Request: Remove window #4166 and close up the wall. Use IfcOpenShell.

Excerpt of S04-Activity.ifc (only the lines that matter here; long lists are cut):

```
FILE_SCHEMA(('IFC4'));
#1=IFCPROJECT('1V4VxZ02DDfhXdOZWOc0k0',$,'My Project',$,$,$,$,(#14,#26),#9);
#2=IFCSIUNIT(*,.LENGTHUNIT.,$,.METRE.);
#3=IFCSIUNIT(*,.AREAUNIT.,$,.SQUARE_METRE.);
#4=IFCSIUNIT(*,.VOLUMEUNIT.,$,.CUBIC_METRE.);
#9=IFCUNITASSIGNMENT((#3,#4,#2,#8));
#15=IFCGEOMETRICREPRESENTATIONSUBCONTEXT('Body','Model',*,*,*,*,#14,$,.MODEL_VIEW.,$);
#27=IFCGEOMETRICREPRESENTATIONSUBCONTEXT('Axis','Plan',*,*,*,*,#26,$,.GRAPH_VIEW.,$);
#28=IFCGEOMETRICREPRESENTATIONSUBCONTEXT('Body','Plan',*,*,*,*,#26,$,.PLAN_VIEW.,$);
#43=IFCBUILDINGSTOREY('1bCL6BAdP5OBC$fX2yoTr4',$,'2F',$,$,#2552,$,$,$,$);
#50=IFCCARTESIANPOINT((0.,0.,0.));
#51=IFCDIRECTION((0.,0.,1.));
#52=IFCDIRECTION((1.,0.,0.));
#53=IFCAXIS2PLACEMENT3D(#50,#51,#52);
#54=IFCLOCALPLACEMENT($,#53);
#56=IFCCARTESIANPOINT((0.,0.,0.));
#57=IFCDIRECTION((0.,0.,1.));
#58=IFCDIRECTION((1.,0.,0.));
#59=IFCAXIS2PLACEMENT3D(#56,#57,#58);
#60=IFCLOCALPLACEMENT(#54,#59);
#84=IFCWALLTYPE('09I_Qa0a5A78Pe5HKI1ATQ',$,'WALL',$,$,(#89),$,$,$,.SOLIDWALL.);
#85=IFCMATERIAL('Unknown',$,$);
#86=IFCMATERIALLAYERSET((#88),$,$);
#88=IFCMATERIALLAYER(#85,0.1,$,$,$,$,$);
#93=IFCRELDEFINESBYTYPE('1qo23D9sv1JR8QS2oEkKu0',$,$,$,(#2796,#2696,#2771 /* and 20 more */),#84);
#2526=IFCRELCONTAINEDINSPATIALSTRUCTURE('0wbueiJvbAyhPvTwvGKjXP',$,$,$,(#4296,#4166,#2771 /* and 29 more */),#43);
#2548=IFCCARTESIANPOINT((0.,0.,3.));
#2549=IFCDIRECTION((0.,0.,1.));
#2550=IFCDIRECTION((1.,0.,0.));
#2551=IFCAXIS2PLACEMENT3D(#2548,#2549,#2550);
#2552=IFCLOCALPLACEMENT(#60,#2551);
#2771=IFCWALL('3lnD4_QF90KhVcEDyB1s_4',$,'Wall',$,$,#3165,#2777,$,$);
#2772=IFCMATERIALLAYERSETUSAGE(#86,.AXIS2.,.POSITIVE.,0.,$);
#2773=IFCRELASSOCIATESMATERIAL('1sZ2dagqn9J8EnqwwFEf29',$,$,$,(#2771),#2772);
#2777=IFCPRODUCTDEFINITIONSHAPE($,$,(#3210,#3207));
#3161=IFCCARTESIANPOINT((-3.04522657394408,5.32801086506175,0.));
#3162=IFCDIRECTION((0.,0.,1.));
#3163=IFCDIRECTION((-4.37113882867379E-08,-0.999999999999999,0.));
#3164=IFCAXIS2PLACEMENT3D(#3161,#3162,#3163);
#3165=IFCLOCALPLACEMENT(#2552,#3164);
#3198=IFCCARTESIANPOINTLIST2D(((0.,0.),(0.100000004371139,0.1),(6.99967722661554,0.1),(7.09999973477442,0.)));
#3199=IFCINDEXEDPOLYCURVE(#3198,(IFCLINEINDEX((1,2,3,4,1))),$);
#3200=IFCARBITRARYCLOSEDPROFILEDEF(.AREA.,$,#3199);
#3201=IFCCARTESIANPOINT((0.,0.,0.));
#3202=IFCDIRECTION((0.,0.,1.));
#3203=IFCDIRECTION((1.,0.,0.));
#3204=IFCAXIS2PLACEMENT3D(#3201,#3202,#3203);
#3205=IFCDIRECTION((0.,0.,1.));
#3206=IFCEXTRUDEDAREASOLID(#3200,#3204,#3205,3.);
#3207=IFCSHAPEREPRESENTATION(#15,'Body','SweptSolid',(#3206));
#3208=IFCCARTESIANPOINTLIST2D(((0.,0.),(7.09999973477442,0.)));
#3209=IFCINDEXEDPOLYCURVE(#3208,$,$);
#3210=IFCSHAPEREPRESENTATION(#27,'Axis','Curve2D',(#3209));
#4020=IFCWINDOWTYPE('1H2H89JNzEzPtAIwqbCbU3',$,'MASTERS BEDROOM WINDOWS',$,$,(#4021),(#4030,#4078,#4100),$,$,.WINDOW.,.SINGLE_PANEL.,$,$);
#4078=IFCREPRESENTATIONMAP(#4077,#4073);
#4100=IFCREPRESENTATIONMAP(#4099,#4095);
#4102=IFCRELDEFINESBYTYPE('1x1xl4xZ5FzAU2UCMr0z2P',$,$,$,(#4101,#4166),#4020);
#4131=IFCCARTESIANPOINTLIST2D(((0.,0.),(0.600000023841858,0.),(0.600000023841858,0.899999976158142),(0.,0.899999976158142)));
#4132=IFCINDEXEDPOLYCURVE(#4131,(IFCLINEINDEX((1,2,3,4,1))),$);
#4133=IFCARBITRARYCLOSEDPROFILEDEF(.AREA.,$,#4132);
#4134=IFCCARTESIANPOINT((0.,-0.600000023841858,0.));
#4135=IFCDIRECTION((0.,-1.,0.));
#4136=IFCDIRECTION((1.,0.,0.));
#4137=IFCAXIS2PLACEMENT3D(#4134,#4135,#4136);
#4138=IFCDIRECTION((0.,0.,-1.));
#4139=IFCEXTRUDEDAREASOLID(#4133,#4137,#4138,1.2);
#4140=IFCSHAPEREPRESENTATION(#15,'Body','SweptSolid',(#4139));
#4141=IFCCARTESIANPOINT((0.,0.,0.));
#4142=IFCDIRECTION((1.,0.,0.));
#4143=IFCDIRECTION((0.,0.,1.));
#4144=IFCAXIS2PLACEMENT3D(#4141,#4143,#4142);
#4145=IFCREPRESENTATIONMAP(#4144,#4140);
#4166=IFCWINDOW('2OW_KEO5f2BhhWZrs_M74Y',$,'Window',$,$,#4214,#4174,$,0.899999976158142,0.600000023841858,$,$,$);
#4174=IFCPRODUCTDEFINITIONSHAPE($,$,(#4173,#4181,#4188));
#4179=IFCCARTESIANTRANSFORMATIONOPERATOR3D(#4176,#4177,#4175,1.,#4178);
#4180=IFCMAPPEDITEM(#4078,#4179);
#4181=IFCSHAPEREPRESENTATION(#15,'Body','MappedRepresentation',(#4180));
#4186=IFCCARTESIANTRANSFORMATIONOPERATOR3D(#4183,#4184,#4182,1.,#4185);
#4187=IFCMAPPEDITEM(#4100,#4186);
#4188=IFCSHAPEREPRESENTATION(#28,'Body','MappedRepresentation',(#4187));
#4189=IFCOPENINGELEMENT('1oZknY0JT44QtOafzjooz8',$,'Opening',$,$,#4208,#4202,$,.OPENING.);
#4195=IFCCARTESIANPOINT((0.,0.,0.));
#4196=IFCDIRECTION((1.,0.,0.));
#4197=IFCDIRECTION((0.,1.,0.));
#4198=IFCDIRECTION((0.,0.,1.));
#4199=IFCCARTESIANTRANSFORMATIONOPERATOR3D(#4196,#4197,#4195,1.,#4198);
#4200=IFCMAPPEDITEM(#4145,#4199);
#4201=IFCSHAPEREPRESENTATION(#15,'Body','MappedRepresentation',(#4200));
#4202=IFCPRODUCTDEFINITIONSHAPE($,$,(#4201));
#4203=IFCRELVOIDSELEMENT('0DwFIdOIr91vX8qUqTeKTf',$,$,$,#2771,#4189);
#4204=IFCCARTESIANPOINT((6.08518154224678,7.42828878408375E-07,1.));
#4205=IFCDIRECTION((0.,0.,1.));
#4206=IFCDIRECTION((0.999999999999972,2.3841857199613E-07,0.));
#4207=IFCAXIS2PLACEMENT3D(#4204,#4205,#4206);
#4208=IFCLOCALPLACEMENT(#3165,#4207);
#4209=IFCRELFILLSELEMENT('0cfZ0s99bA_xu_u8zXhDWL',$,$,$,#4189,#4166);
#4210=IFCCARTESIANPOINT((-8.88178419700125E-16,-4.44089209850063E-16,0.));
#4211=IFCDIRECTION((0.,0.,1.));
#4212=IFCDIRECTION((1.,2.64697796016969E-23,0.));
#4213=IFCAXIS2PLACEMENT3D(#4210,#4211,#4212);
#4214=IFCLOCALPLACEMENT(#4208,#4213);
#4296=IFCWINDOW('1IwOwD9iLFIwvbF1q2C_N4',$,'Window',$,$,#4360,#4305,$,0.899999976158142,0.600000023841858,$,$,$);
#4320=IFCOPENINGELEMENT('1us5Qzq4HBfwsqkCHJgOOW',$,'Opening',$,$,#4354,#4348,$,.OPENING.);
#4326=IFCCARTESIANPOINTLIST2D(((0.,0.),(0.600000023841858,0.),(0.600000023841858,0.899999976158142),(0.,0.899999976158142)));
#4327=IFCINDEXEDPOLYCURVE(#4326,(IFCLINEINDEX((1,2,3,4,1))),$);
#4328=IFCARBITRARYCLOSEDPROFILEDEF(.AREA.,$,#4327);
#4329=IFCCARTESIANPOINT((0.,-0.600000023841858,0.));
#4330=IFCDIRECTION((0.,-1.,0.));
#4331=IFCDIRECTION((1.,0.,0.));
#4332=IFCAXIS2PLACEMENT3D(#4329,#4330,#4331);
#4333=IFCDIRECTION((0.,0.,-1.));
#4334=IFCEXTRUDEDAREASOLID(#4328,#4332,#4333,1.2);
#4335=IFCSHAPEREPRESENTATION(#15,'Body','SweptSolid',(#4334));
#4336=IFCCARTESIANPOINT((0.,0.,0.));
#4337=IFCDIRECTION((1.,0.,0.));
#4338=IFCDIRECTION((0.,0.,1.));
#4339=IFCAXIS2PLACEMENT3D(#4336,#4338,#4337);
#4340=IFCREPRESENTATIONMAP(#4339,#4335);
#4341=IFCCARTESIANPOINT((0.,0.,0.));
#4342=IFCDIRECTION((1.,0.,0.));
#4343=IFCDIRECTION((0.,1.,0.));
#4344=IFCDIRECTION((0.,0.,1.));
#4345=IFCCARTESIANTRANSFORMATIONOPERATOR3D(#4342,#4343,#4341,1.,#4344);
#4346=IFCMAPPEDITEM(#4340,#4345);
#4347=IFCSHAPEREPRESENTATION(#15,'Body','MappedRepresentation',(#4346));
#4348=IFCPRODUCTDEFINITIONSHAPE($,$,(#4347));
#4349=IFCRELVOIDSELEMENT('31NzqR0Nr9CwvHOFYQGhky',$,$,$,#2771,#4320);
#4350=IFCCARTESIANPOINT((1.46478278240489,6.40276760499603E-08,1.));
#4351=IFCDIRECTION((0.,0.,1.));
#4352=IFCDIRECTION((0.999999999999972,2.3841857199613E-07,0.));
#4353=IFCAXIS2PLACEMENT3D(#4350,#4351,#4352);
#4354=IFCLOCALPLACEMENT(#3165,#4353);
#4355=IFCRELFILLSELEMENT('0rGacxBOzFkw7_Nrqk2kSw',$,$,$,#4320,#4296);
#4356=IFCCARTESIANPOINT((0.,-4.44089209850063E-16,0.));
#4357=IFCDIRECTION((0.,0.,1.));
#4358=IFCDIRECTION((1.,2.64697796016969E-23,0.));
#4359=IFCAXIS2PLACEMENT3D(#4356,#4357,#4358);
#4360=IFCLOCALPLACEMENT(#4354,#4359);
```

```python
import ifcopenshell
import ifcopenshell.api.feature
import ifcopenshell.api.root
import ifcopenshell.geom
import ifcopenshell.util.shape

model = ifcopenshell.open("S04-Activity.ifc")
settings = ifcopenshell.geom.settings()


def volume(element):
    """Net volume in cubic metres, openings subtracted."""
    shape = ifcopenshell.geom.create_shape(settings, element)
    return ifcopenshell.util.shape.get_volume(shape.geometry)


window = model.by_guid("2OW_KEO5f2BhhWZrs_M74Y")
opening = window.FillsVoids[0].RelatingOpeningElement
wall = opening.VoidsElements[0].RelatingBuildingElement
before = volume(wall)

ifcopenshell.api.root.remove_product(model, product=window)
ifcopenshell.api.feature.remove_feature(model, feature=opening)

after = volume(wall)

print(f"wall volume {before:.3f} -> {after:.3f} m3")

model.write("S04-Activity_edited.ifc")
```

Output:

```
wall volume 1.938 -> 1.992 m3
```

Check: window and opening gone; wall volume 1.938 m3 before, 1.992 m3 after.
